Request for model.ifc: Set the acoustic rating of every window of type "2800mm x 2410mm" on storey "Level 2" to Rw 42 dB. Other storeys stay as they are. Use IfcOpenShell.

First a look at what the model holds.

```python
import ifcopenshell
import ifcopenshell.util.element

model = ifcopenshell.open("model.ifc")
print(model.schema)
storey = next(s for s in model.by_type("IfcBuildingStorey") if s.Name == "Level 2")
windows = [e for e in ifcopenshell.util.element.get_decomposition(storey) if e.is_a("IfcWindow")]
seen = {}
for e in windows:
    element_type = ifcopenshell.util.element.get_type(e)
    key = (element_type.Name if element_type != e and element_type else None, ifcopenshell.util.element.get_pset(e, "Pset_WindowCommon", "AcousticRating"))
    seen[key] = seen.get(key, 0) + 1
for (name, value), count in sorted(seen.items(), key=str):
    print(count, "x", name, "|", value)
```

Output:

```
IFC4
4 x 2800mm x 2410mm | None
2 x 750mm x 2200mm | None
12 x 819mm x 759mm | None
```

```python
import ifcopenshell
import ifcopenshell.api.pset
import ifcopenshell.util.element

model = ifcopenshell.open("model.ifc")

storey = next(s for s in model.by_type("IfcBuildingStorey") if s.Name == "Level 2")
windows = [e for e in ifcopenshell.util.element.get_decomposition(storey) if e.is_a("IfcWindow")]

count = 0
for e in windows:
    element_type = ifcopenshell.util.element.get_type(e)
    if element_type in (None, e) or element_type.Name != "2800mm x 2410mm":
        continue
    # add_pset returns the element's existing set when there is one.
    pset = ifcopenshell.api.pset.add_pset(model, product=e, name="Pset_WindowCommon")
    ifcopenshell.api.pset.edit_pset(model, pset=pset, properties={"AcousticRating": "Rw 42 dB"})
    count += 1

print(count, "windows updated")

model.write("model-out.ifc")
```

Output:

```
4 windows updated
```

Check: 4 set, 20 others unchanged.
